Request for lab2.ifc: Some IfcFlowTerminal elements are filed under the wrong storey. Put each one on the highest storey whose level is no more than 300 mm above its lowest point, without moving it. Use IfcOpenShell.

First a look at what the model holds.

```python
import ifcopenshell
import ifcopenshell.util.element
import ifcopenshell.util.placement

model = ifcopenshell.open("lab2.ifc")
print(model.schema)
for storey in model.by_type("IfcBuildingStorey"):
    level = ifcopenshell.util.placement.get_storey_elevation(storey)
    count = sum(e.is_a("IfcFlowTerminal") for e in ifcopenshell.util.element.get_contained(storey))
    print(storey.id(), storey.Name, round(level, 3), count, sep=" | ")
```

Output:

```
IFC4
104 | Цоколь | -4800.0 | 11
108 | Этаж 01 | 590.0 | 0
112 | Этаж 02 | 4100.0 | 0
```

```python
import ifcopenshell
import ifcopenshell.api.spatial
import ifcopenshell.geom
import ifcopenshell.util.element
import ifcopenshell.util.placement
import ifcopenshell.util.shape
import ifcopenshell.util.unit

model = ifcopenshell.open("lab2.ifc")
unit_scale = ifcopenshell.util.unit.calculate_unit_scale(model)
settings = ifcopenshell.geom.settings()

levels = sorted(
    ((ifcopenshell.util.placement.get_storey_elevation(s) * unit_scale, s) for s in model.by_type("IfcBuildingStorey")),
    key=lambda pair: pair[0],
)

for e in model.by_type("IfcFlowTerminal"):
    current = e.ContainedInStructure[0].RelatingStructure if e.ContainedInStructure else None
    if current is None or not current.is_a("IfcBuildingStorey"):
        continue
    shape = ifcopenshell.geom.create_shape(settings, e)
    bottom = ifcopenshell.util.shape.get_shape_bottom_elevation(shape, shape.geometry)
    below = [s for level, s in levels if level <= bottom + 0.3]
    storey = below[-1] if below else levels[0][1]
    if storey != current:
        # assign_container keeps the world position.
        ifcopenshell.api.spatial.assign_container(model, products=[e], relating_structure=storey)
        print(e.id(), current.Name, "->", storey.Name)

model.write("lab2_updated.ifc")
```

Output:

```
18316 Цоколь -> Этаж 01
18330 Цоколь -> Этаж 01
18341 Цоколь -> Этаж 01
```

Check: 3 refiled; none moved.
